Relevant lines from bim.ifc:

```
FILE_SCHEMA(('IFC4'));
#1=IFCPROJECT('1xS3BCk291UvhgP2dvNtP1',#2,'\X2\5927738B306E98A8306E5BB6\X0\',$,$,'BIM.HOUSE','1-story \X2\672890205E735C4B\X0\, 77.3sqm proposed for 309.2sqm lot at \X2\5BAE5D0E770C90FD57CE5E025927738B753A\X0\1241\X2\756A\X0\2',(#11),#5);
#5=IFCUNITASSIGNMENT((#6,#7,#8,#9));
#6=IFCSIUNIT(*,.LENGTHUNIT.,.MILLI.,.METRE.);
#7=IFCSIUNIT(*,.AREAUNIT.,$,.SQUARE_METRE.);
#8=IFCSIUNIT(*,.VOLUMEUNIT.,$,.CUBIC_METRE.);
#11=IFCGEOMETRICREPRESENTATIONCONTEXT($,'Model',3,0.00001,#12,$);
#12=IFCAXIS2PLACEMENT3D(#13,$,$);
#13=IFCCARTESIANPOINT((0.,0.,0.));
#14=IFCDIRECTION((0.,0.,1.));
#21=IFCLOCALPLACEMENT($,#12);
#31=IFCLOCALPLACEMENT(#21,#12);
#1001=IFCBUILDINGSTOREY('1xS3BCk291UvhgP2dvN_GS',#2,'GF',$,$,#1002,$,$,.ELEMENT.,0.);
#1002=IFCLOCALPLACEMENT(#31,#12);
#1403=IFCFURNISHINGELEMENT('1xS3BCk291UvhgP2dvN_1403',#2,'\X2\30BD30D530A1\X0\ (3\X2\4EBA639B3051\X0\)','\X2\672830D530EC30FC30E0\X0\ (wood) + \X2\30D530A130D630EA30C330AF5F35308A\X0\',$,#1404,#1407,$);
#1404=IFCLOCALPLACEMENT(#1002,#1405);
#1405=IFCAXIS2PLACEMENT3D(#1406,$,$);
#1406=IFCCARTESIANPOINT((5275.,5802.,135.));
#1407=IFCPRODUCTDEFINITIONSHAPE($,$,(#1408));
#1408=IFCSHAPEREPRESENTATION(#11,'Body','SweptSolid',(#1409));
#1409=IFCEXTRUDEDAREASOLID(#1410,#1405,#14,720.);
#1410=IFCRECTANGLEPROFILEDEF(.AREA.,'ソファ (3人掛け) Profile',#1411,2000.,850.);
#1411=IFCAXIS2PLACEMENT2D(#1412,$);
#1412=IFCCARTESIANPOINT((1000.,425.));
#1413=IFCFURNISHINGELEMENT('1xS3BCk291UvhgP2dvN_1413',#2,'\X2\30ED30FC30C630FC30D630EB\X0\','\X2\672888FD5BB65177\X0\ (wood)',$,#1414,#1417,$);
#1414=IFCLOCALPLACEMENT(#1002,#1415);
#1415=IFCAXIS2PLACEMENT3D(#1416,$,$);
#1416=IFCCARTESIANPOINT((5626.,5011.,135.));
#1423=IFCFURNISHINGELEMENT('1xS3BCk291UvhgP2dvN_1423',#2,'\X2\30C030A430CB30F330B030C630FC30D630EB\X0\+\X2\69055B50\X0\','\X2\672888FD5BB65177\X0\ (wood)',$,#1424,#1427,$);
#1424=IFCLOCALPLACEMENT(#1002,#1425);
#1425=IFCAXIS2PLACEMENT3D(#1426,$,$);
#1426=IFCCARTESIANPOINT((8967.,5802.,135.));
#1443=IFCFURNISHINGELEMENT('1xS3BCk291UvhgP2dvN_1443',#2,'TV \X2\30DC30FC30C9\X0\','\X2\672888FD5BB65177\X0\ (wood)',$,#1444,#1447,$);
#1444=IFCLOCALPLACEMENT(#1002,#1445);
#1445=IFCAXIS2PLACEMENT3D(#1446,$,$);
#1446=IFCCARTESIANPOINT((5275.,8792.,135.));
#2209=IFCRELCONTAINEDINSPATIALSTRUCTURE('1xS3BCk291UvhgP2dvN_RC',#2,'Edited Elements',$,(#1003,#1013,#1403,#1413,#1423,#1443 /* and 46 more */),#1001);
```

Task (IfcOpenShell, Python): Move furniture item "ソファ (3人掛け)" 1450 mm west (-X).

```python
import ifcopenshell
import ifcopenshell.api.geometry
import ifcopenshell.util.placement
import ifcopenshell.util.unit

model = ifcopenshell.open("bim.ifc")
unit_scale = ifcopenshell.util.unit.calculate_unit_scale(model)

item = model.by_guid("1xS3BCk291UvhgP2dvN_1403")
matrix = ifcopenshell.util.placement.get_local_placement(item.ObjectPlacement)
matrix[0, 3] -= 1.45 / unit_scale
ifcopenshell.api.geometry.edit_object_placement(model, product=item, matrix=matrix, is_si=False)

print(ifcopenshell.util.placement.get_local_placement(item.ObjectPlacement).round(3) + 0.0)

model.write("bim_updated.ifc")
```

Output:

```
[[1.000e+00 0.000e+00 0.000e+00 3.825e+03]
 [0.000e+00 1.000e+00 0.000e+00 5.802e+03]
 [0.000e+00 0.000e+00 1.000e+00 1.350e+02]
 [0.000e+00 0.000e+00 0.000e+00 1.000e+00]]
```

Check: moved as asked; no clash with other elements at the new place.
